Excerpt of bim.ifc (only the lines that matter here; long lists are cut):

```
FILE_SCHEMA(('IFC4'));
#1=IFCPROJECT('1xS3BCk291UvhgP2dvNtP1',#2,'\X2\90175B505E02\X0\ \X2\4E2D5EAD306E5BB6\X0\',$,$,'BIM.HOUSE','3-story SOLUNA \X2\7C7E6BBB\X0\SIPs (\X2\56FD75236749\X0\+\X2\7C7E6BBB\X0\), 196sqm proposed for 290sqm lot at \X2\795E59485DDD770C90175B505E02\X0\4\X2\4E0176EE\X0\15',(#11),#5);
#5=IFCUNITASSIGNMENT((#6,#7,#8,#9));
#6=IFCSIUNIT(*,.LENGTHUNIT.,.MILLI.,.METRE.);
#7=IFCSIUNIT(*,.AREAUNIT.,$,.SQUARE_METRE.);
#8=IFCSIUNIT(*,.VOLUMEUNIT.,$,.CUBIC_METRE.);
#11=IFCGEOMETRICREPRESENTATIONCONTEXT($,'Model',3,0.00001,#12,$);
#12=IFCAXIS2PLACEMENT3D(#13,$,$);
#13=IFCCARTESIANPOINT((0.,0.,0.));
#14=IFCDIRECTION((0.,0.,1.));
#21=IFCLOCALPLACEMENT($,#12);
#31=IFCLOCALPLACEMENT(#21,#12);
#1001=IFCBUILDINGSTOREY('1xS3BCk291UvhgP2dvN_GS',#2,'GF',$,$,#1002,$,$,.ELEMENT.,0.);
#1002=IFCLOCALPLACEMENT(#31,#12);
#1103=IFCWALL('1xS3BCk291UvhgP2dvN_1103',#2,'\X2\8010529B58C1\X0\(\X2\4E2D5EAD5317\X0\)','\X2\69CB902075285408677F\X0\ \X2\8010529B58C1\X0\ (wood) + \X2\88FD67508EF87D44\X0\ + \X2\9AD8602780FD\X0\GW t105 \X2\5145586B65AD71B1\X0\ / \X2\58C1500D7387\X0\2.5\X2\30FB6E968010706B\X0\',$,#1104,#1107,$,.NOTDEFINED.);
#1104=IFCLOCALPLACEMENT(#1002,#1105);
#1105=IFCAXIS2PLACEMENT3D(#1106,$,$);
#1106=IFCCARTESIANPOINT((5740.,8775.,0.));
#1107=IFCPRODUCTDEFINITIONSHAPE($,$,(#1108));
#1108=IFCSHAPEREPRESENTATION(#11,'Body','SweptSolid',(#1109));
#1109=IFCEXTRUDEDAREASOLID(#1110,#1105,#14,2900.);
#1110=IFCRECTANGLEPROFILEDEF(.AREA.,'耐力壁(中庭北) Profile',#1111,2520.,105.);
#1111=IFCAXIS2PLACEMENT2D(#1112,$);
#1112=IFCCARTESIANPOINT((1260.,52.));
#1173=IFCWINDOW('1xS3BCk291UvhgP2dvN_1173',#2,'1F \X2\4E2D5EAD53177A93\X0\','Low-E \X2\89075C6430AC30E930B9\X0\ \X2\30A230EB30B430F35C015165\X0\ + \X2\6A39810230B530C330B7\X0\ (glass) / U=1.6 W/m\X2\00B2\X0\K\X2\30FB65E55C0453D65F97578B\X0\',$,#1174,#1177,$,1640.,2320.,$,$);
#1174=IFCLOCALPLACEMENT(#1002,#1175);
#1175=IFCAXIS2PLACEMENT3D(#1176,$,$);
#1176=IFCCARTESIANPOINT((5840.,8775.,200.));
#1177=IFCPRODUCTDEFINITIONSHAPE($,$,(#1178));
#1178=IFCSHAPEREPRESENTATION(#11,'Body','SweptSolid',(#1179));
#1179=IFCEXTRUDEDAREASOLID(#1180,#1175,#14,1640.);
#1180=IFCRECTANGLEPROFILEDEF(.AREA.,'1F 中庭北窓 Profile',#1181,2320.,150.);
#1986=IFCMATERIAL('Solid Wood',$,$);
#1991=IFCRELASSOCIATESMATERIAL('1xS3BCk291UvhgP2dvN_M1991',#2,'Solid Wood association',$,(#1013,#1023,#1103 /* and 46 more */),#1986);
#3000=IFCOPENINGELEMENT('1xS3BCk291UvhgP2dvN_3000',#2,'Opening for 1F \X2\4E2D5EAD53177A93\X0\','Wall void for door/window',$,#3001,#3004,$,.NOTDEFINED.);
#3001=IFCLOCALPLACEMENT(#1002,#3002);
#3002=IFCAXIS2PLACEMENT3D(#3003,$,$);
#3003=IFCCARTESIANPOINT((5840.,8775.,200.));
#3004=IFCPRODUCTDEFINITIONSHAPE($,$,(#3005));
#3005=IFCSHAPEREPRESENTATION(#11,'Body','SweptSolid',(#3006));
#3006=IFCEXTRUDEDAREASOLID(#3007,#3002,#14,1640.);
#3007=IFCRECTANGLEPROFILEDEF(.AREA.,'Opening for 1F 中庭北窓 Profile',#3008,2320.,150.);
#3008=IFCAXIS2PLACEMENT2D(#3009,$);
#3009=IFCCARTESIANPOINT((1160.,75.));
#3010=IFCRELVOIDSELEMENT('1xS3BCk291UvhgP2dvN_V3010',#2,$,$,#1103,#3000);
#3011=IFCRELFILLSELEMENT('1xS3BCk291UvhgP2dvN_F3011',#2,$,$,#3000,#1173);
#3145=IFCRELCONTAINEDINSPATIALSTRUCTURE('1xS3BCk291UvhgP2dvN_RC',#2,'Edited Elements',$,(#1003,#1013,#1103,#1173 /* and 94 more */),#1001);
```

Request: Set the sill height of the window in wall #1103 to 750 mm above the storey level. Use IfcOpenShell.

```python
import numpy as np
import ifcopenshell
import ifcopenshell.api.geometry
import ifcopenshell.geom
import ifcopenshell.util.element
import ifcopenshell.util.placement
import ifcopenshell.util.shape
import ifcopenshell.util.unit

model = ifcopenshell.open("bim.ifc")
unit_scale = ifcopenshell.util.unit.calculate_unit_scale(model)

window = model.by_guid("1xS3BCk291UvhgP2dvN_1173")
opening = window.FillsVoids[0].RelatingOpeningElement
storey = ifcopenshell.util.element.get_container(window, ifc_class="IfcBuildingStorey")
level = ifcopenshell.util.placement.get_local_placement(storey.ObjectPlacement)[2, 3]

# The opening's origin need not be at the sill, so measure its lowest point.
shape = ifcopenshell.geom.create_shape(ifcopenshell.geom.settings(), opening)
bottom = ifcopenshell.util.shape.get_shape_bottom_elevation(shape, shape.geometry) / unit_scale
dz = level + 750.0 - bottom

shift = np.array([0.0, 0.0, dz])
# The window is not placed relative to its opening, so move both.
for product in (opening, window):
    matrix = ifcopenshell.util.placement.get_local_placement(product.ObjectPlacement)
    matrix[:3, 3] += shift
    ifcopenshell.api.geometry.edit_object_placement(model, product=product, matrix=matrix, is_si=False)

print(f"moved by {dz * unit_scale:+.3f} m")

model.write("bim_updated.ifc")
```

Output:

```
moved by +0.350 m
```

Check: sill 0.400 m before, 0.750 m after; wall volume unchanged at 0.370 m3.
